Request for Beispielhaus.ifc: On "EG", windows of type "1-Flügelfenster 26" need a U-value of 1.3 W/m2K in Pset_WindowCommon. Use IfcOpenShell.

First a look at what the model holds.

```python
import ifcopenshell
import ifcopenshell.util.element

model = ifcopenshell.open("Beispielhaus.ifc")
print(model.schema)
storey = next(s for s in model.by_type("IfcBuildingStorey") if s.Name == "EG")
windows = [e for e in ifcopenshell.util.element.get_decomposition(storey) if e.is_a("IfcWindow")]
seen = {}
for e in windows:
    element_type = ifcopenshell.util.element.get_type(e)
    key = (element_type.Name if element_type != e and element_type else None, ifcopenshell.util.element.get_pset(e, "Pset_WindowCommon", "ThermalTransmittance"))
    seen[key] = seen.get(key, 0) + 1
for (name, value), count in sorted(seen.items(), key=str):
    print(count, "x", name, "|", value)
```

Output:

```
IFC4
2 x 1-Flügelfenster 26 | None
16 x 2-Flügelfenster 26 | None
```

```python
import ifcopenshell
import ifcopenshell.api.pset
import ifcopenshell.util.element

model = ifcopenshell.open("Beispielhaus.ifc")

storey = next(s for s in model.by_type("IfcBuildingStorey") if s.Name == "EG")
windows = [e for e in ifcopenshell.util.element.get_decomposition(storey) if e.is_a("IfcWindow")]

count = 0
for e in windows:
    element_type = ifcopenshell.util.element.get_type(e)
    if element_type in (None, e) or element_type.Name != "1-Flügelfenster 26":
        continue
    # add_pset returns the element's existing set when there is one.
    pset = ifcopenshell.api.pset.add_pset(model, product=e, name="Pset_WindowCommon")
    ifcopenshell.api.pset.edit_pset(model, pset=pset, properties={"ThermalTransmittance": 1.3})
    count += 1

print(count, "windows updated")

model.write("Beispielhaus-out.ifc")
```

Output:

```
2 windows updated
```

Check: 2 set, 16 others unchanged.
